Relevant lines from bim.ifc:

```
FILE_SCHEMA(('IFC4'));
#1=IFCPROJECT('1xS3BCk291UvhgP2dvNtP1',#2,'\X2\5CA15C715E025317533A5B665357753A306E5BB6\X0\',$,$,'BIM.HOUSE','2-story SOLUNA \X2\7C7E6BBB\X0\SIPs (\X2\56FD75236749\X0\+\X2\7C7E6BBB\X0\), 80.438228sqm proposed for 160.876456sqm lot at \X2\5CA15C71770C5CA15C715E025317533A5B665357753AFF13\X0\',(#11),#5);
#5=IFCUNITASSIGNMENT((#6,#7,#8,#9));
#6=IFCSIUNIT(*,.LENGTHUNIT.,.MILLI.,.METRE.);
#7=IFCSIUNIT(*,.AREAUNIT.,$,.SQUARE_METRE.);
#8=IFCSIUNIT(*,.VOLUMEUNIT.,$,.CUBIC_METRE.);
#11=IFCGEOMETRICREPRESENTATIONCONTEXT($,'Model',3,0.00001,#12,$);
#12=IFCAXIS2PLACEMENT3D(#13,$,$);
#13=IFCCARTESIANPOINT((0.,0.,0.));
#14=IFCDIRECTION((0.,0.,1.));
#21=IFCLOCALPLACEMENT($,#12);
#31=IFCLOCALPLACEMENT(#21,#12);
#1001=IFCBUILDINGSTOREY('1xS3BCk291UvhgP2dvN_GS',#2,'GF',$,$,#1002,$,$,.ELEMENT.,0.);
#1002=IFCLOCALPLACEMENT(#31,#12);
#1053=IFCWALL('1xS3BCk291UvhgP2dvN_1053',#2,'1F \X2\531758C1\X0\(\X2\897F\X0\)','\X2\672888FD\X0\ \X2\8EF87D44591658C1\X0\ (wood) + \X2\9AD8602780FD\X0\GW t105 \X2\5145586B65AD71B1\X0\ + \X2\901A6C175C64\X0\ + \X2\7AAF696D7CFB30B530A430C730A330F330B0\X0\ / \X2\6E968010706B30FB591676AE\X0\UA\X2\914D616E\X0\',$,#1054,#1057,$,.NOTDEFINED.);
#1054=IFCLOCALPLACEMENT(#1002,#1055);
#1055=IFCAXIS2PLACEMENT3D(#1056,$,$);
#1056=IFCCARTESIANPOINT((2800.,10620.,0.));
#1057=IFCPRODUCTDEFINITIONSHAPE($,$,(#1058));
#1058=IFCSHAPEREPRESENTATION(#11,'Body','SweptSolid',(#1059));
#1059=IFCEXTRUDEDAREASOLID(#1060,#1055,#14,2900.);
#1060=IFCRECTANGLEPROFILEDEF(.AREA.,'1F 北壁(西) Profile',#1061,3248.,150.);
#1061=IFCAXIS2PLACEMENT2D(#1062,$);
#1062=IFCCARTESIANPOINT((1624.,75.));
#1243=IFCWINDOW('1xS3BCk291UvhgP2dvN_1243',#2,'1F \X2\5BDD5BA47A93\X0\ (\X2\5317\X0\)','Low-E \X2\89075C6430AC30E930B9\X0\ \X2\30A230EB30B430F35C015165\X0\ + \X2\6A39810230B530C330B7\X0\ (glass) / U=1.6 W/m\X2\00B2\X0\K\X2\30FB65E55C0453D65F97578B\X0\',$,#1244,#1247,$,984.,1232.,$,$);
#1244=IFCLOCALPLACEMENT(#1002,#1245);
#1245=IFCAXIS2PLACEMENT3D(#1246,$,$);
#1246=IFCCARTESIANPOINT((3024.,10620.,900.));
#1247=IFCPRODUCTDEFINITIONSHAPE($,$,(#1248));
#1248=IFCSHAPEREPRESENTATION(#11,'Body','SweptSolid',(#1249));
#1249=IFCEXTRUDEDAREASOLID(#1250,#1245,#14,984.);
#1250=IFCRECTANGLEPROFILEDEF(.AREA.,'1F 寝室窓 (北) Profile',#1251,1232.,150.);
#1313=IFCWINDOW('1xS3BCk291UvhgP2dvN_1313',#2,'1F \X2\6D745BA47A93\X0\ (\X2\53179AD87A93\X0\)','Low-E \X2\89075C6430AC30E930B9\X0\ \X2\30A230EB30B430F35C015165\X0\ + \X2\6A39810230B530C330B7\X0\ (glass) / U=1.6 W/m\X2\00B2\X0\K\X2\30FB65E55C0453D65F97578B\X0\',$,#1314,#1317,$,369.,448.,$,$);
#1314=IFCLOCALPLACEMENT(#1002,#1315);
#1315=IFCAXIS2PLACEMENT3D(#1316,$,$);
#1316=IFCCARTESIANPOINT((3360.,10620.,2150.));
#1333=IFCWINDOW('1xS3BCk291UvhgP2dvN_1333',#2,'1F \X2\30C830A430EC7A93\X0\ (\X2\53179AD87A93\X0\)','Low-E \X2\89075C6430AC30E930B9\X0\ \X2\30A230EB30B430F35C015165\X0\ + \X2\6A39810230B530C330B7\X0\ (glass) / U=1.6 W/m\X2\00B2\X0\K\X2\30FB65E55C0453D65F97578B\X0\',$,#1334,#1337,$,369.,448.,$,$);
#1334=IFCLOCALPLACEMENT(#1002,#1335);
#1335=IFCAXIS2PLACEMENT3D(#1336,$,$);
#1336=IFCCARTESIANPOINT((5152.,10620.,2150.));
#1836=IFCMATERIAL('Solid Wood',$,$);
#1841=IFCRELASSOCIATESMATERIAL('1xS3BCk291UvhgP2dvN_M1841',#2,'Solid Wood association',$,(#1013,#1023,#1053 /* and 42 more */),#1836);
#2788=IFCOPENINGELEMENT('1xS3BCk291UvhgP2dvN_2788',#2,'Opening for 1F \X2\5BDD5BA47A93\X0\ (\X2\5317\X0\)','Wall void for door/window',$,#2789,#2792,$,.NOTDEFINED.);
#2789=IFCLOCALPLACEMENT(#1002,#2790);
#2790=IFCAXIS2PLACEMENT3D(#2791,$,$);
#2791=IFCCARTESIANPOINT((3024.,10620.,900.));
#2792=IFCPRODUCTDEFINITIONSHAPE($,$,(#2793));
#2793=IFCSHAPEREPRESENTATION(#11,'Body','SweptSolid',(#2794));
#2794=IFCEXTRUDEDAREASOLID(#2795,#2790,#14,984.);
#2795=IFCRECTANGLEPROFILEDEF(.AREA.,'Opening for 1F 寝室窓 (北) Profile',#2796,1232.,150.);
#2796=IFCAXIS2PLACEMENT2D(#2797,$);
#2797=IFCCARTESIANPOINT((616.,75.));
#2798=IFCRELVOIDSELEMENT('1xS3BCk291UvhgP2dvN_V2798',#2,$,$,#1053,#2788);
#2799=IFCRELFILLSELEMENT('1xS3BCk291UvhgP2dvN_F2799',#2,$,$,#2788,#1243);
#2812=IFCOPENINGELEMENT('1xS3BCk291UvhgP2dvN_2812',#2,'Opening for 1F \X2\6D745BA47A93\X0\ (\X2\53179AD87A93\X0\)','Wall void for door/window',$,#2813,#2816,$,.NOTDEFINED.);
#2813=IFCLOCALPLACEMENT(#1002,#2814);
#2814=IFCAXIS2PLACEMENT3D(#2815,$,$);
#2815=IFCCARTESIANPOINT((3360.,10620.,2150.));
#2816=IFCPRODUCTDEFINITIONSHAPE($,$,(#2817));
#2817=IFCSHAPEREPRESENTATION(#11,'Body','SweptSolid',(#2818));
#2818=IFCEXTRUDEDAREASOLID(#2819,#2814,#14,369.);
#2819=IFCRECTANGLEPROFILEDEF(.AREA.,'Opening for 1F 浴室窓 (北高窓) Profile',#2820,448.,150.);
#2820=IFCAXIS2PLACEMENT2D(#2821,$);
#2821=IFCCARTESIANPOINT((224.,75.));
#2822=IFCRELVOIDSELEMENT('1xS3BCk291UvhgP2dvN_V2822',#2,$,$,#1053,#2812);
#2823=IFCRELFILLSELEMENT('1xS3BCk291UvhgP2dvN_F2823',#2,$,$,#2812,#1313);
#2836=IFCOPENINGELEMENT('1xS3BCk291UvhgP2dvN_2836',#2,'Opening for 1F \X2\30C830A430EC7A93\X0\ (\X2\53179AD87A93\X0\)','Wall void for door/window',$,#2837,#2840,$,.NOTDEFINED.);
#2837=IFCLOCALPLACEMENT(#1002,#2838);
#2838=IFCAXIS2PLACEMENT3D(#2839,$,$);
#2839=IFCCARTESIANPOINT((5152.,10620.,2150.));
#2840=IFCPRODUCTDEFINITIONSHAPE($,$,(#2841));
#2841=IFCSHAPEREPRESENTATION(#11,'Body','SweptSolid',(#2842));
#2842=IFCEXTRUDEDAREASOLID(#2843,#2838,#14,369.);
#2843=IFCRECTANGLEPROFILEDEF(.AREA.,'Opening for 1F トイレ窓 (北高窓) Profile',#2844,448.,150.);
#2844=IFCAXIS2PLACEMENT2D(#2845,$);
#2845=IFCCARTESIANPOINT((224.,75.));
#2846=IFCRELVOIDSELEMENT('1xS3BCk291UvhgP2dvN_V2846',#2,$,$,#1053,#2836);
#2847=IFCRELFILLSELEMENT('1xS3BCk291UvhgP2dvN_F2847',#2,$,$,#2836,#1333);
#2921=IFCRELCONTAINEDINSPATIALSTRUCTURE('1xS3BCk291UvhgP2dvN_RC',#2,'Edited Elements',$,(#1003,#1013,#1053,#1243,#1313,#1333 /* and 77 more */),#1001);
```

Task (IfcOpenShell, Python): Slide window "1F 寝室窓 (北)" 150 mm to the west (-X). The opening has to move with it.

```python
import ifcopenshell
import ifcopenshell.api.geometry
import ifcopenshell.util.placement

model = ifcopenshell.open("bim.ifc")

window = model.by_guid("1xS3BCk291UvhgP2dvN_1243")
opening = window.FillsVoids[0].RelatingOpeningElement
wall = opening.VoidsElements[0].RelatingBuildingElement

wall_matrix = ifcopenshell.util.placement.get_local_placement(wall.ObjectPlacement)
shift = wall_matrix[:3, 0] * -150.0
before = ifcopenshell.util.placement.get_local_placement(window.ObjectPlacement)[:3, 3].copy()

# The window is not placed relative to its opening, so move both.
for product in (opening, window):
    matrix = ifcopenshell.util.placement.get_local_placement(product.ObjectPlacement)
    matrix[:3, 3] += shift
    ifcopenshell.api.geometry.edit_object_placement(model, product=product, matrix=matrix, is_si=False)

after = ifcopenshell.util.placement.get_local_placement(window.ObjectPlacement)[:3, 3]
print("window moved by", (after - before).round(3) + 0.0)

model.write("bim-out.ifc")
```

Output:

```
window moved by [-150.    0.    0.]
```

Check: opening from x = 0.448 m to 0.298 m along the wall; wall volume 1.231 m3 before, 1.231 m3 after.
